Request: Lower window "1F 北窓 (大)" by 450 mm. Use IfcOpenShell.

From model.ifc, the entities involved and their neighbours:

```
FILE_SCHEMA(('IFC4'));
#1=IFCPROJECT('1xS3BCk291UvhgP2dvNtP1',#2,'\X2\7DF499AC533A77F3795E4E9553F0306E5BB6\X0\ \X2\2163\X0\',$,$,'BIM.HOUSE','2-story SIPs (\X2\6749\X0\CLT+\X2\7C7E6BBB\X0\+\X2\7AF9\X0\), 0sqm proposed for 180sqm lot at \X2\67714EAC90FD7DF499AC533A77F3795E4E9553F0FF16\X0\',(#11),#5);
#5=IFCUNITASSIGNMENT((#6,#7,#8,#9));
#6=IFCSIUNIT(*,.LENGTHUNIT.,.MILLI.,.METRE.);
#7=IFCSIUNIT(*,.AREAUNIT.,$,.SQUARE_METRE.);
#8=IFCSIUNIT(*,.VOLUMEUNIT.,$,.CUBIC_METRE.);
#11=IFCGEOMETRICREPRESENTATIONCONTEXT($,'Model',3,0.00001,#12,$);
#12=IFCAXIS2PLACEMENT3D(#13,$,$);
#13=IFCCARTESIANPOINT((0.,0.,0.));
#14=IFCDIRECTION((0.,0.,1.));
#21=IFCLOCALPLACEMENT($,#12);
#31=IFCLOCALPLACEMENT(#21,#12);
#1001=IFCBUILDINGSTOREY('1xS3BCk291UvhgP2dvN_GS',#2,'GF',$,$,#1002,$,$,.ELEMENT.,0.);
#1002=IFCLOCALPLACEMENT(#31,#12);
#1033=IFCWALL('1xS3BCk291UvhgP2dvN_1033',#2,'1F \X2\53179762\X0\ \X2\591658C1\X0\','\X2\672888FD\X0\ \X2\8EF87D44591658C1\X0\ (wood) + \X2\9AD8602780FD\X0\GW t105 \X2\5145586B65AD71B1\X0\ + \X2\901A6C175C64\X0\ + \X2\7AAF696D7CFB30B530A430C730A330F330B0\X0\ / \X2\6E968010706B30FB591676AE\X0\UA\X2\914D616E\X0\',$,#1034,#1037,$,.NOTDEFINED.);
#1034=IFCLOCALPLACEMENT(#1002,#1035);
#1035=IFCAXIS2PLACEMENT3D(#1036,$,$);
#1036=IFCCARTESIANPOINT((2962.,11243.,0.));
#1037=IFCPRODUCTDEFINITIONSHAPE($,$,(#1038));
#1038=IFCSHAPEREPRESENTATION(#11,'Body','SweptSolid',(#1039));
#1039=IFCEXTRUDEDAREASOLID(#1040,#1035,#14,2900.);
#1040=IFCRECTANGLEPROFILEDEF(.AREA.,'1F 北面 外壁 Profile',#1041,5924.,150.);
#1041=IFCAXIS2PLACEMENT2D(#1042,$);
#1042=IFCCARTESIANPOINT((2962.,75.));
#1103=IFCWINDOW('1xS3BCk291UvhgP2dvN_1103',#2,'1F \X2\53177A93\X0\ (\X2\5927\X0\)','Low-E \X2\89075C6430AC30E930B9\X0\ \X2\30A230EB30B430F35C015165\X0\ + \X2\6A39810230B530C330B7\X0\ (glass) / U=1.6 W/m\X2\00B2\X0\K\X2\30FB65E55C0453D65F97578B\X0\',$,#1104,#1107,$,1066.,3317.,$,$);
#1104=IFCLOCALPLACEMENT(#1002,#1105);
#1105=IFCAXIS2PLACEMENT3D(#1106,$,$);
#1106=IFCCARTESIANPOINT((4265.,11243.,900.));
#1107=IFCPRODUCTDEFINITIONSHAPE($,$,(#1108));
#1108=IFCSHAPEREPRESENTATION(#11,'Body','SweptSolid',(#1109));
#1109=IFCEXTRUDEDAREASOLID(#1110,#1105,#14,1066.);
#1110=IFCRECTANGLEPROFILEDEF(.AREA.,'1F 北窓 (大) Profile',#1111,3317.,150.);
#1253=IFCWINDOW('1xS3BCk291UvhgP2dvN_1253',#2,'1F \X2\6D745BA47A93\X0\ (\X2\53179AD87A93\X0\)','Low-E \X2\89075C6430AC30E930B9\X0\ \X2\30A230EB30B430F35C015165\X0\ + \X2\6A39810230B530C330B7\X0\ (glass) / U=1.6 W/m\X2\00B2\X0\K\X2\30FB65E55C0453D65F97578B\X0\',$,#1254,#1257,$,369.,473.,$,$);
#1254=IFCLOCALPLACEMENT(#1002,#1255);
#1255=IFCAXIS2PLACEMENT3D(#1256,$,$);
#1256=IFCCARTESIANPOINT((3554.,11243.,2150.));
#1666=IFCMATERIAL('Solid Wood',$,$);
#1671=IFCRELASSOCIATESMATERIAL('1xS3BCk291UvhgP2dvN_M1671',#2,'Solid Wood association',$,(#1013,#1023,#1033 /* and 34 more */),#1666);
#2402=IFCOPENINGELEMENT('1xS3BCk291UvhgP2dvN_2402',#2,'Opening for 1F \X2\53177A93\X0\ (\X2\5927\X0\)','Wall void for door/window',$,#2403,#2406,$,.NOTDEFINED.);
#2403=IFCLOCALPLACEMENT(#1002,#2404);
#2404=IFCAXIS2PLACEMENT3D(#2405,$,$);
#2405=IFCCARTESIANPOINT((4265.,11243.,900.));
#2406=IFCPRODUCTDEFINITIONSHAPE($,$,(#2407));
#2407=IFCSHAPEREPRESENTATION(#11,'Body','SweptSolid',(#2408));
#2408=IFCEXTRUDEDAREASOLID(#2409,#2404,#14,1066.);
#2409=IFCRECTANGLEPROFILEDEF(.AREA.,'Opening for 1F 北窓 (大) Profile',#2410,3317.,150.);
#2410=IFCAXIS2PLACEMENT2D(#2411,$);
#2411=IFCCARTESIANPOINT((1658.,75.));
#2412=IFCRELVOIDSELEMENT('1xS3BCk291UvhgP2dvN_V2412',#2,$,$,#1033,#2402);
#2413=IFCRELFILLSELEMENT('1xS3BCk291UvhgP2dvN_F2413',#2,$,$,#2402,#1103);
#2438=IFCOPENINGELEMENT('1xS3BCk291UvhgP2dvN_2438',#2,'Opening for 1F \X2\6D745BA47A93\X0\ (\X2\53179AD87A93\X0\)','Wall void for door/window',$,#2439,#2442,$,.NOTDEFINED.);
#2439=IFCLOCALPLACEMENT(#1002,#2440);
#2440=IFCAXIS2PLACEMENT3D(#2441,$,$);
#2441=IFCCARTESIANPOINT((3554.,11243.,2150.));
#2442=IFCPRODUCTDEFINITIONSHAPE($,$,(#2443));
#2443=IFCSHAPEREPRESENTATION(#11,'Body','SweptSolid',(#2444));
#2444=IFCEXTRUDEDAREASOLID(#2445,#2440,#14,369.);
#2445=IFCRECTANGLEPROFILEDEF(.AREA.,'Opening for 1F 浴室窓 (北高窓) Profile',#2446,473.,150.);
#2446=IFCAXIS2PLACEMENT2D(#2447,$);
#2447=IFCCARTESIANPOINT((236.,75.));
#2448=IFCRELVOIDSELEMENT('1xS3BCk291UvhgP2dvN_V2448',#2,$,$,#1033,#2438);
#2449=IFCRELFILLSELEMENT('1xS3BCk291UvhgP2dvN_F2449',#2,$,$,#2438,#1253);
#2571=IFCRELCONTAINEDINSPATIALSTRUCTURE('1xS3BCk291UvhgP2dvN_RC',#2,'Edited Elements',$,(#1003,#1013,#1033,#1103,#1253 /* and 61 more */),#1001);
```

```python
import numpy as np
import ifcopenshell
import ifcopenshell.api.geometry
import ifcopenshell.util.placement
import ifcopenshell.util.unit

model = ifcopenshell.open("model.ifc")
unit_scale = ifcopenshell.util.unit.calculate_unit_scale(model)

window = model.by_guid("1xS3BCk291UvhgP2dvN_1103")
opening = window.FillsVoids[0].RelatingOpeningElement
dz = -0.45 / unit_scale

shift = np.array([0.0, 0.0, dz])
# The window is not placed relative to its opening, so move both.
for product in (opening, window):
    matrix = ifcopenshell.util.placement.get_local_placement(product.ObjectPlacement)
    matrix[:3, 3] += shift
    ifcopenshell.api.geometry.edit_object_placement(model, product=product, matrix=matrix, is_si=False)

print(f"moved by {dz * unit_scale:+.3f} m")

model.write("model_rev.ifc")
```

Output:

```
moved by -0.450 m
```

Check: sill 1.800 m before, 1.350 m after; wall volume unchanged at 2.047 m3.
